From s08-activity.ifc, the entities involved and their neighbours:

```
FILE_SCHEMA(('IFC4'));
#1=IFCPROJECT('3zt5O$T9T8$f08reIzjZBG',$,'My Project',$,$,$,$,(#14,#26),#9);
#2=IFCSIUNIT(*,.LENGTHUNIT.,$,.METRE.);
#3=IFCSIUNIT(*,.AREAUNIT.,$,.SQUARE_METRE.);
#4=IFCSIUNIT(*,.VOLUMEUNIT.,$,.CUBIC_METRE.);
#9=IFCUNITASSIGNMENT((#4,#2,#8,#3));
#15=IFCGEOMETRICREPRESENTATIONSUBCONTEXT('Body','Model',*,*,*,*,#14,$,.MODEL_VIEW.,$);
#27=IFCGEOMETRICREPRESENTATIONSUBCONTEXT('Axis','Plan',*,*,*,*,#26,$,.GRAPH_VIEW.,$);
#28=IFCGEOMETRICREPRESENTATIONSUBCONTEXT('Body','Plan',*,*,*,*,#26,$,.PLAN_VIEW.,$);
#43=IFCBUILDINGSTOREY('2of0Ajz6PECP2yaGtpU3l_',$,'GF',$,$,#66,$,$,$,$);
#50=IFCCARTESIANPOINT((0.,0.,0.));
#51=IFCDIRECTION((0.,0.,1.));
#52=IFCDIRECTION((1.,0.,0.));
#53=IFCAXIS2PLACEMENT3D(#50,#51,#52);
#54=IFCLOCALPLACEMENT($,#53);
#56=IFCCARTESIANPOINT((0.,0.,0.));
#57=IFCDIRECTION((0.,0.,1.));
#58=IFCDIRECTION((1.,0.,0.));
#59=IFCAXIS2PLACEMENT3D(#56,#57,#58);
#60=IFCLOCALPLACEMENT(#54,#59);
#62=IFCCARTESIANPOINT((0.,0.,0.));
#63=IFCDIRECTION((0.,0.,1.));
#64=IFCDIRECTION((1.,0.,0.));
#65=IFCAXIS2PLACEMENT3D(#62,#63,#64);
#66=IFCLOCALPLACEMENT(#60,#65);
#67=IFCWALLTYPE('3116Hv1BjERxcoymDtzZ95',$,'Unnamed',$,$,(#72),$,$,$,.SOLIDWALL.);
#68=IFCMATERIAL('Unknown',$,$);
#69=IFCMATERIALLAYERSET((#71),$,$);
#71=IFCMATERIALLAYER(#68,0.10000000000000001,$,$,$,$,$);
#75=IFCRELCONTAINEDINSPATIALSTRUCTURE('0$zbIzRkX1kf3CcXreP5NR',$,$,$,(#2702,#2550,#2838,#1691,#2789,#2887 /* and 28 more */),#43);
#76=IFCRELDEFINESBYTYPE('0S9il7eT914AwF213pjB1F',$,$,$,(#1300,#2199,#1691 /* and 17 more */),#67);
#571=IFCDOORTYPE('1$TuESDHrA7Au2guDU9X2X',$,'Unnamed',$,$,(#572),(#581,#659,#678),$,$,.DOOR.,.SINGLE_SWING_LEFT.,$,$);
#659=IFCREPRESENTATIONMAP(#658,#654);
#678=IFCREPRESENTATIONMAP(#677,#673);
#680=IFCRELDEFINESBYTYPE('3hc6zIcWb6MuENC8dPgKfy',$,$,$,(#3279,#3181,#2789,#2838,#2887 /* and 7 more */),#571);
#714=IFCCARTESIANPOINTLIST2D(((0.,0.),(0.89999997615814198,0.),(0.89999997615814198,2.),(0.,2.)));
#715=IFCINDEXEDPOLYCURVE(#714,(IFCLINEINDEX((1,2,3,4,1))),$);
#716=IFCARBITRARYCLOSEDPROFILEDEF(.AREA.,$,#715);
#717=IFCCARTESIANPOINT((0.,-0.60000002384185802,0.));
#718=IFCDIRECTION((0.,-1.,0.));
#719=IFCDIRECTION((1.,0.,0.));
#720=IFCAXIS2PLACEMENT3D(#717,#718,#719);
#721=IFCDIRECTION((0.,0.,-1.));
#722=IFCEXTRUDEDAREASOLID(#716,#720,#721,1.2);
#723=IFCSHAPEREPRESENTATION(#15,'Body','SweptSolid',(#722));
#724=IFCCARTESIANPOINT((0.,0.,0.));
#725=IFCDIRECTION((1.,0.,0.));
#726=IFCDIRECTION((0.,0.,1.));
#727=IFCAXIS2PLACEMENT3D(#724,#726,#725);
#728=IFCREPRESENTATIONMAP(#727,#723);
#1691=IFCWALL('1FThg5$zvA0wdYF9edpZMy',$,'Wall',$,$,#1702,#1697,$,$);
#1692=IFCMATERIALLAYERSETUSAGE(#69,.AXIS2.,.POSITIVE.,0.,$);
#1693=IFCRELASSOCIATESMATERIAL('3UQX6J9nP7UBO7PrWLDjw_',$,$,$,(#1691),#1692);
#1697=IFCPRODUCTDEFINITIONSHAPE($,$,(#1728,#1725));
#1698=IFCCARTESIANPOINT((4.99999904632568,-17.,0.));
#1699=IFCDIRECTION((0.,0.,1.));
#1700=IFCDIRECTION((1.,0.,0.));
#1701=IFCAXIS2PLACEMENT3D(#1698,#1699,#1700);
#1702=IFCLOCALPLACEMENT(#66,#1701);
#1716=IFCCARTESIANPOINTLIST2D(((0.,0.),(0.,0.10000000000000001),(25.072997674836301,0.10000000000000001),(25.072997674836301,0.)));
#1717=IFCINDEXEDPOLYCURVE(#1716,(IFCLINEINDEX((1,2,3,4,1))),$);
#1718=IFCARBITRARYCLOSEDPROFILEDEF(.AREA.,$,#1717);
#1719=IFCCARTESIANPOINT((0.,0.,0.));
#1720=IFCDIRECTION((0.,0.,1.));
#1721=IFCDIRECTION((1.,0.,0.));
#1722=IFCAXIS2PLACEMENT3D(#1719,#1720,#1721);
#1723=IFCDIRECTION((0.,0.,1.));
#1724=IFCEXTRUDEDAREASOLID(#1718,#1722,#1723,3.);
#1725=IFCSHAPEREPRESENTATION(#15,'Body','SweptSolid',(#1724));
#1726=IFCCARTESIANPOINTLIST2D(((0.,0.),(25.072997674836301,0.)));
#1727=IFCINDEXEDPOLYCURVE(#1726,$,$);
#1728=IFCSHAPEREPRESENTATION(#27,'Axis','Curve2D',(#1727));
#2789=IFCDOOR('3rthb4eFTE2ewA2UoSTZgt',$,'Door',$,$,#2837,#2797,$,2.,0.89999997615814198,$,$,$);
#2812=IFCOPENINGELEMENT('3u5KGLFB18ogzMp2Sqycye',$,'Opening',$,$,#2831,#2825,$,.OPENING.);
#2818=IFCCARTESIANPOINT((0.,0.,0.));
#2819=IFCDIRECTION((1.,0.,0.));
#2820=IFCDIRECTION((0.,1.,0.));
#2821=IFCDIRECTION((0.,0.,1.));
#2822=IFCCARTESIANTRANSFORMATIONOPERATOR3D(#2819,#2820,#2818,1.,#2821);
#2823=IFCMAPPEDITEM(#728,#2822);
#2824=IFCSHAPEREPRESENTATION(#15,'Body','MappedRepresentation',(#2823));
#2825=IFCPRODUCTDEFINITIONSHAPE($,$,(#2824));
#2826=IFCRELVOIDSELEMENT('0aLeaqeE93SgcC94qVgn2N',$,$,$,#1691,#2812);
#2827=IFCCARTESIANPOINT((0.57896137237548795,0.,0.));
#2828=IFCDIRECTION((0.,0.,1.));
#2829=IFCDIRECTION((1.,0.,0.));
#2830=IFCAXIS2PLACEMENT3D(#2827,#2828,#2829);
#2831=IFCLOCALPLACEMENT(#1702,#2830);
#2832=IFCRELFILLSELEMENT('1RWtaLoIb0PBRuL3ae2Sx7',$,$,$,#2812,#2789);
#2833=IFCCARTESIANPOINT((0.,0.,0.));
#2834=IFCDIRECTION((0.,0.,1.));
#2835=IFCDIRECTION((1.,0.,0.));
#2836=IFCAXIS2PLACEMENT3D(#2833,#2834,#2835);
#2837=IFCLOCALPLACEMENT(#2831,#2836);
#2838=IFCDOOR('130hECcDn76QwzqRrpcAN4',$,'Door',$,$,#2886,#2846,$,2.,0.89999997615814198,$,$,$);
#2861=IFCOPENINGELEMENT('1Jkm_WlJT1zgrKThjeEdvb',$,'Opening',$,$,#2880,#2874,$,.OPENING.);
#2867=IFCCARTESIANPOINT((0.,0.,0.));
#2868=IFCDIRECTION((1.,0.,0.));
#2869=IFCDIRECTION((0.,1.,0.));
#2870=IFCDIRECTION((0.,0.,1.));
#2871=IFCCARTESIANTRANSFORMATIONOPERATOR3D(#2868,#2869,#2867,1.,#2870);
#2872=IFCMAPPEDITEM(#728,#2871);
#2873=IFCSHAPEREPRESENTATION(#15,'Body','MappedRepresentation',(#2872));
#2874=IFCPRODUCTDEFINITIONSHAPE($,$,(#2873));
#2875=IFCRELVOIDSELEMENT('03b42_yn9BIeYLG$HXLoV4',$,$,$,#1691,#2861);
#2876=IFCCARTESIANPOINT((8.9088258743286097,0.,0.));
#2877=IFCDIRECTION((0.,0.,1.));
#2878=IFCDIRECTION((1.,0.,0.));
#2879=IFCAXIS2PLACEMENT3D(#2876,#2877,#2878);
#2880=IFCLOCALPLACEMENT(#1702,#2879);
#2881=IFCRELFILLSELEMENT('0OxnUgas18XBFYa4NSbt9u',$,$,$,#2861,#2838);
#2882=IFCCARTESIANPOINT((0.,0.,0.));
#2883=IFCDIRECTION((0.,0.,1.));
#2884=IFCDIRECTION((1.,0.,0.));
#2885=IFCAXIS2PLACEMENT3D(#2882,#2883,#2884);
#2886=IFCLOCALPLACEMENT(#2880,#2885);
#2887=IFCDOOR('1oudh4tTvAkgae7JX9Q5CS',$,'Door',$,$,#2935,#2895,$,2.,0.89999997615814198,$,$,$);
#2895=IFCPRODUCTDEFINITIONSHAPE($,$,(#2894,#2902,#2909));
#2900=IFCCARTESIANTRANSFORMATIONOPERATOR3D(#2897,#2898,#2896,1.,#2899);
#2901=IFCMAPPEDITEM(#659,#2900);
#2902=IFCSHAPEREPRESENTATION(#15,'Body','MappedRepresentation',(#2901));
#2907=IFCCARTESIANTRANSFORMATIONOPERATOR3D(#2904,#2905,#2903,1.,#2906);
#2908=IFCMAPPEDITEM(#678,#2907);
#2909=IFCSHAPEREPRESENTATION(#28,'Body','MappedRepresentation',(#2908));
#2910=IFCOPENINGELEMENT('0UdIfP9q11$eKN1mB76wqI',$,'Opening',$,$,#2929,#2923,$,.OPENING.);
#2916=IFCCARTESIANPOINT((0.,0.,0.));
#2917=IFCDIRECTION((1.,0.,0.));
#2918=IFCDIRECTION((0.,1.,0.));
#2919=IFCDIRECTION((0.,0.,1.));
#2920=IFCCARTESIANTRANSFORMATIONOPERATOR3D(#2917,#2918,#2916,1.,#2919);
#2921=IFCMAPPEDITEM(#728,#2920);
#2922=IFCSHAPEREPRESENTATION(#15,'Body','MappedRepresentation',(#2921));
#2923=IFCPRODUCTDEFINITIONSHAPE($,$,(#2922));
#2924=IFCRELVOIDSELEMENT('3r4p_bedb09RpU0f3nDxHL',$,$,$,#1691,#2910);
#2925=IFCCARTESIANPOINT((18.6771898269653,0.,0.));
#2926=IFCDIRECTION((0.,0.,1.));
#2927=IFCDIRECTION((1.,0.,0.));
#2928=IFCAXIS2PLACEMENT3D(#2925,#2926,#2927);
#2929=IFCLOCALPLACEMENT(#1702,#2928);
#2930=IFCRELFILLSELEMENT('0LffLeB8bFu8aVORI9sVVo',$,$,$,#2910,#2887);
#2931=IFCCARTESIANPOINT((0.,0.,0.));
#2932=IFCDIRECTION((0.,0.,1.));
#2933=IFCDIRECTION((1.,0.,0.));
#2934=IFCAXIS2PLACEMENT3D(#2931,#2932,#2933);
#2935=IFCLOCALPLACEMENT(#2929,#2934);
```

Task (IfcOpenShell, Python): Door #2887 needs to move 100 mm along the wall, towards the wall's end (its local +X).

```python
import ifcopenshell
import ifcopenshell.api.geometry
import ifcopenshell.util.placement
import ifcopenshell.util.unit

model = ifcopenshell.open("s08-activity.ifc")
unit_scale = ifcopenshell.util.unit.calculate_unit_scale(model)

door = model.by_guid("1oudh4tTvAkgae7JX9Q5CS")
opening = door.FillsVoids[0].RelatingOpeningElement
wall = opening.VoidsElements[0].RelatingBuildingElement

wall_matrix = ifcopenshell.util.placement.get_local_placement(wall.ObjectPlacement)
shift = wall_matrix[:3, 0] * 0.1 / unit_scale
before = ifcopenshell.util.placement.get_local_placement(door.ObjectPlacement)[:3, 3].copy()

# The door is placed relative to its opening, so it follows when the opening moves.
matrix = ifcopenshell.util.placement.get_local_placement(opening.ObjectPlacement)
matrix[:3, 3] += shift
ifcopenshell.api.geometry.edit_object_placement(
    model, product=opening, matrix=matrix, is_si=False, should_transform_children=True
)

after = ifcopenshell.util.placement.get_local_placement(door.ObjectPlacement)[:3, 3]
print("door moved by", (after - before).round(3) + 0.0)

model.write("s08-activity_rev.ifc")
```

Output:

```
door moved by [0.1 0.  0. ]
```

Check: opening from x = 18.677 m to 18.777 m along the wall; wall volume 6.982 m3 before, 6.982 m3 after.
